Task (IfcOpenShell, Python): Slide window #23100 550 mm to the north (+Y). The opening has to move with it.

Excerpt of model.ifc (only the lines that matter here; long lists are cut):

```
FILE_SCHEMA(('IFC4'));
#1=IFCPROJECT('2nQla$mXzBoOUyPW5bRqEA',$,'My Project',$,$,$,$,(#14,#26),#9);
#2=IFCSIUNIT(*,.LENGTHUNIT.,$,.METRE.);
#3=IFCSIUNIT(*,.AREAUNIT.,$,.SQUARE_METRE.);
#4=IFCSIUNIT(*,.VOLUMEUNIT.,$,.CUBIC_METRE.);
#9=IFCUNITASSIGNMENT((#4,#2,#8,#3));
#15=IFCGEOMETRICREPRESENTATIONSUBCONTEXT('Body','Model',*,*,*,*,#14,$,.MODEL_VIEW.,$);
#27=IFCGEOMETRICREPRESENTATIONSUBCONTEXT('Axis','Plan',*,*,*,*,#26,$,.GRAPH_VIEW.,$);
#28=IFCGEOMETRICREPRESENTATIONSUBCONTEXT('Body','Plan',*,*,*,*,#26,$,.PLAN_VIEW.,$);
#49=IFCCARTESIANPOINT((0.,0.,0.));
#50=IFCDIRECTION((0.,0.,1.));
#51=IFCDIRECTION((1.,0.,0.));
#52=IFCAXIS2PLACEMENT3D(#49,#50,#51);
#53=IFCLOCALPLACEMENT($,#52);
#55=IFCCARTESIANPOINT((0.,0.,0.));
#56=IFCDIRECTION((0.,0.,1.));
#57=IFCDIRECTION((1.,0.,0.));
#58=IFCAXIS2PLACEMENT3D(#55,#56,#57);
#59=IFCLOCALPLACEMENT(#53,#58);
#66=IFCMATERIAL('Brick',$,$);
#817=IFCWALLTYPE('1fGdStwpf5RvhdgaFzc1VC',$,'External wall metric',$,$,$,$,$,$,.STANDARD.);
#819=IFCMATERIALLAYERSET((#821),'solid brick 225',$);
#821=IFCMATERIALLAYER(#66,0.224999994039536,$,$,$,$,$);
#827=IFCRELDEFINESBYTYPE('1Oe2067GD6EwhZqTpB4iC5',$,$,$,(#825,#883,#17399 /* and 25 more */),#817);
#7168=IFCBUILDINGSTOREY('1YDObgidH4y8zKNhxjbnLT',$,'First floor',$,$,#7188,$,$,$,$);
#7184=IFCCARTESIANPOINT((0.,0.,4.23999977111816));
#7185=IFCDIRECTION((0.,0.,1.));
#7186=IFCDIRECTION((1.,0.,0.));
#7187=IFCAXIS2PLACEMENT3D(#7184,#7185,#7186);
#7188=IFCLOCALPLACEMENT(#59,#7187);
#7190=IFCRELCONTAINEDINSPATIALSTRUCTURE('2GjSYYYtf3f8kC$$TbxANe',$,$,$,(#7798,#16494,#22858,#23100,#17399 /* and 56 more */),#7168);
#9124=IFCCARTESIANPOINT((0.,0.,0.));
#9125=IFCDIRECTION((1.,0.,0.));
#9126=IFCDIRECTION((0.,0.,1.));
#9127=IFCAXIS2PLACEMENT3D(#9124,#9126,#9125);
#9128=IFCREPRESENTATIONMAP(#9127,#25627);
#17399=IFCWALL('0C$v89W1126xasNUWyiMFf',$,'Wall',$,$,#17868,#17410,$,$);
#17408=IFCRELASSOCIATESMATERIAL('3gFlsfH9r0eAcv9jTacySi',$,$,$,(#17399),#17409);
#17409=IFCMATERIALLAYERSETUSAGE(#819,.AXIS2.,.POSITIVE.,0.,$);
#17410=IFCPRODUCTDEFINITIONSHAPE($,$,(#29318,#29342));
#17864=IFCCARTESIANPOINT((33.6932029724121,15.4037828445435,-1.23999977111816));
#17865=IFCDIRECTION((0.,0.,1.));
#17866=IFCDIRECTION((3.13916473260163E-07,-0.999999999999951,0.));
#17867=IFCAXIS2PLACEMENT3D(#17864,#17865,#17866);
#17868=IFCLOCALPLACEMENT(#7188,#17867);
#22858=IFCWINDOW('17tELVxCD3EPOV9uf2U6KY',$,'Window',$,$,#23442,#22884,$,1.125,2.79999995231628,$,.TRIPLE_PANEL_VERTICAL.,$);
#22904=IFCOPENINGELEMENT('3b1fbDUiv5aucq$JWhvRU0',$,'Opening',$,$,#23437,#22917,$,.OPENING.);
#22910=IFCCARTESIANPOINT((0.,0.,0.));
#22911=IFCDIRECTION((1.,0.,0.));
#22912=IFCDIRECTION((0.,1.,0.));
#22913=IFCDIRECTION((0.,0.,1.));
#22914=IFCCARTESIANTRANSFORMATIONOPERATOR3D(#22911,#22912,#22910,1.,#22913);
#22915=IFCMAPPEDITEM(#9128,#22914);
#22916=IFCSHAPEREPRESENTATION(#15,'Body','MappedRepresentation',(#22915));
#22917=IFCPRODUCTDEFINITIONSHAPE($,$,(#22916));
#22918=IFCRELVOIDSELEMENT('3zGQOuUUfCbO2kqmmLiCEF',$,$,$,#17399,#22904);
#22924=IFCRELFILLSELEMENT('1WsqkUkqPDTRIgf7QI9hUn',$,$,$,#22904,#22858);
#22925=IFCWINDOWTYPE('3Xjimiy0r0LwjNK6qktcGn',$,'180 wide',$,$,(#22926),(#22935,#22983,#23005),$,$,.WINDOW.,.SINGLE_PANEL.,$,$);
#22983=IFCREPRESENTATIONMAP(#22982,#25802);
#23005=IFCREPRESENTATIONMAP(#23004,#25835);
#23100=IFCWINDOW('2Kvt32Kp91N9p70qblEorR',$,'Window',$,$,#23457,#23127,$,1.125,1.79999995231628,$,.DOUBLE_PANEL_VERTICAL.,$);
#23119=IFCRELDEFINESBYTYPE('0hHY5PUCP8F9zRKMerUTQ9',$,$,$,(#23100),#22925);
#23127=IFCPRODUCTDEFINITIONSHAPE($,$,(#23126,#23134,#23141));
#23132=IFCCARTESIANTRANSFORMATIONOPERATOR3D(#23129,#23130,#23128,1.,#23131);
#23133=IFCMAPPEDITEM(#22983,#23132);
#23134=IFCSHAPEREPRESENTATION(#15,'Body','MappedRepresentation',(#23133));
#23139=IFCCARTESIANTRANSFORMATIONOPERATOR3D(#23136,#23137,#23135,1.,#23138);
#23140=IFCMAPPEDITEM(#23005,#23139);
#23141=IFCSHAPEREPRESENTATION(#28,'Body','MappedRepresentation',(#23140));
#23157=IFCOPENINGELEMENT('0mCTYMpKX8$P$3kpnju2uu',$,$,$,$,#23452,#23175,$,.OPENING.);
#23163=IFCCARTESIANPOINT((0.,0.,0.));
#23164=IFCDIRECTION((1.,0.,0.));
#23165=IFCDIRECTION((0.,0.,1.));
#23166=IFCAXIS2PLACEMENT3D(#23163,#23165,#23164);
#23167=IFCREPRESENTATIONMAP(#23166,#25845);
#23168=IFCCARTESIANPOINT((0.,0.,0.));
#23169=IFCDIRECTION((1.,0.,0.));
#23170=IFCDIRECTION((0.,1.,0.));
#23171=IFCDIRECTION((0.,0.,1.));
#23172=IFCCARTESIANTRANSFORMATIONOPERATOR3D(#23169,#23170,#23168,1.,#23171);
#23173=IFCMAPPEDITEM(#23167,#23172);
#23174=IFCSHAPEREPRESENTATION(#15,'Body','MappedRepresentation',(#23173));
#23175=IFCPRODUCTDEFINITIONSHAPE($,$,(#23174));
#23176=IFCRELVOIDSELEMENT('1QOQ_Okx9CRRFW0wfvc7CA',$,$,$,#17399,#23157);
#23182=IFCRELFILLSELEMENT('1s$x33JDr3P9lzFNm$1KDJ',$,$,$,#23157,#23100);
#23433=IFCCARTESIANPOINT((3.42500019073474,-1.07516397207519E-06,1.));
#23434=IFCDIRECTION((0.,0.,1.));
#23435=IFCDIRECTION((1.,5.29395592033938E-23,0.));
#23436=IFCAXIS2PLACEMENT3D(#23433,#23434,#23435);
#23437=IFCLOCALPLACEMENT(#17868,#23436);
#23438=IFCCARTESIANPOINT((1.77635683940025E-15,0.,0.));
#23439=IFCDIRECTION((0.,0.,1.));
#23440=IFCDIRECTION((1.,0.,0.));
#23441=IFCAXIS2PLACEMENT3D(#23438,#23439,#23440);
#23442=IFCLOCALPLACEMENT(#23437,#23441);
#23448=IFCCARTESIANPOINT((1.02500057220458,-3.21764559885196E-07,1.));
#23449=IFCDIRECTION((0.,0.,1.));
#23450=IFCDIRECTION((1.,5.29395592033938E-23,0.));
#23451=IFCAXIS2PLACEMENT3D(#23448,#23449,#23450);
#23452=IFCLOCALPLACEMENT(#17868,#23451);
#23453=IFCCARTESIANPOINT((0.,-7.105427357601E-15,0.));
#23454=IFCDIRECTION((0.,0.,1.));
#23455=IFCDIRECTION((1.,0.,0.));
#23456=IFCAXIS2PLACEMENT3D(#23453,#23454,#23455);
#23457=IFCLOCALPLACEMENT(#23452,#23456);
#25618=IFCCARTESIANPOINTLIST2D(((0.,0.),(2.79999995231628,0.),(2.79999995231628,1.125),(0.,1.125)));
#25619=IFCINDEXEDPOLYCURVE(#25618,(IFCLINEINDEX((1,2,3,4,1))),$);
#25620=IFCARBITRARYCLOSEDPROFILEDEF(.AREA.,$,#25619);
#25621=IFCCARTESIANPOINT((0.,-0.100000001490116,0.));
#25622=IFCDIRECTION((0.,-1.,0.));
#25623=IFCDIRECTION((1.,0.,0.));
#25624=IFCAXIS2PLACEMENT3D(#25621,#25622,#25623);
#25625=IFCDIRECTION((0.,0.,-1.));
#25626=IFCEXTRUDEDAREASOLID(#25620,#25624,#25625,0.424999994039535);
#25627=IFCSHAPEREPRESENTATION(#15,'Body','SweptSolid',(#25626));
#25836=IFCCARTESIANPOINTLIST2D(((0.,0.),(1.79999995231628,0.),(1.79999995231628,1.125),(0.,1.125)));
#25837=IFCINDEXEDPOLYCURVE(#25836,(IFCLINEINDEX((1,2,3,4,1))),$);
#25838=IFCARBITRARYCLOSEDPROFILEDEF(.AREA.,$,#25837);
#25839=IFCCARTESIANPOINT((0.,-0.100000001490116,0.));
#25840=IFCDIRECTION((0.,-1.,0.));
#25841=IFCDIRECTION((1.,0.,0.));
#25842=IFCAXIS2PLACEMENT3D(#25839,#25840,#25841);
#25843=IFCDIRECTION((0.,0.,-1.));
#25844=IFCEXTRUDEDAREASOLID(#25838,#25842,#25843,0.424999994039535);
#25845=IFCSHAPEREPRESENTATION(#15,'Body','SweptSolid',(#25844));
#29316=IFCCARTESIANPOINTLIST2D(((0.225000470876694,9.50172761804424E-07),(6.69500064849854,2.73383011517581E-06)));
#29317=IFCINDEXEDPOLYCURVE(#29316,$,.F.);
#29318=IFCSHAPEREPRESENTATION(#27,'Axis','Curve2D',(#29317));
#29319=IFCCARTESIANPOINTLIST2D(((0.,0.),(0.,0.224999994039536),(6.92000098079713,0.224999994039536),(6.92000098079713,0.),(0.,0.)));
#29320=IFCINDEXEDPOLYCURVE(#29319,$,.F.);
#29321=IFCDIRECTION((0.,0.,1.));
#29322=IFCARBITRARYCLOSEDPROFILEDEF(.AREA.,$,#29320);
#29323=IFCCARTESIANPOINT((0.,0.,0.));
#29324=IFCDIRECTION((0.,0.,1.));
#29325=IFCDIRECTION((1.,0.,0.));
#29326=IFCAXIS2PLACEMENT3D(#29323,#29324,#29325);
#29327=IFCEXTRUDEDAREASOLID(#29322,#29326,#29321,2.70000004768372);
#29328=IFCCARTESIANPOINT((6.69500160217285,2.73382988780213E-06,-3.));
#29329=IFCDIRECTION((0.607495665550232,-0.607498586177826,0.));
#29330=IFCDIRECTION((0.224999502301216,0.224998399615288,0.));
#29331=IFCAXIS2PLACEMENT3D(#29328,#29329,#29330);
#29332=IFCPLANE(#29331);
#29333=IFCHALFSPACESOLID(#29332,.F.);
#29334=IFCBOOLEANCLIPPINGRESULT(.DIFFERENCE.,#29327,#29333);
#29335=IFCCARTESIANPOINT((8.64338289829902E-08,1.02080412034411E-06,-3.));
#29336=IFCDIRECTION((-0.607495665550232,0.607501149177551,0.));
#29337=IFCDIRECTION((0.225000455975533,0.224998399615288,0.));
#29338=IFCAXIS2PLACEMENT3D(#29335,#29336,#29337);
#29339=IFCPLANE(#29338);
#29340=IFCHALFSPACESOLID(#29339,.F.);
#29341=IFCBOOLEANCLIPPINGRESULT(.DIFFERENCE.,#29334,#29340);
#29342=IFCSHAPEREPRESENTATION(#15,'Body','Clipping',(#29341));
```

```python
import ifcopenshell
import ifcopenshell.api.geometry
import ifcopenshell.util.placement
import ifcopenshell.util.unit

model = ifcopenshell.open("model.ifc")
unit_scale = ifcopenshell.util.unit.calculate_unit_scale(model)

window = model.by_id(23100)
opening = window.FillsVoids[0].RelatingOpeningElement
wall = opening.VoidsElements[0].RelatingBuildingElement

wall_matrix = ifcopenshell.util.placement.get_local_placement(wall.ObjectPlacement)
shift = wall_matrix[:3, 0] * -0.55 / unit_scale
before = ifcopenshell.util.placement.get_local_placement(window.ObjectPlacement)[:3, 3].copy()

# The window is placed relative to its opening, so it follows when the opening moves.
matrix = ifcopenshell.util.placement.get_local_placement(opening.ObjectPlacement)
matrix[:3, 3] += shift
ifcopenshell.api.geometry.edit_object_placement(
    model, product=opening, matrix=matrix, is_si=False, should_transform_children=True
)

after = ifcopenshell.util.placement.get_local_placement(window.ObjectPlacement)[:3, 3]
print("window moved by", (after - before).round(3) + 0.0)

model.write("model_v2.ifc")
```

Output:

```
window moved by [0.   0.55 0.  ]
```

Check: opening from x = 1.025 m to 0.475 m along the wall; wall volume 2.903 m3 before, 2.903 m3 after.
